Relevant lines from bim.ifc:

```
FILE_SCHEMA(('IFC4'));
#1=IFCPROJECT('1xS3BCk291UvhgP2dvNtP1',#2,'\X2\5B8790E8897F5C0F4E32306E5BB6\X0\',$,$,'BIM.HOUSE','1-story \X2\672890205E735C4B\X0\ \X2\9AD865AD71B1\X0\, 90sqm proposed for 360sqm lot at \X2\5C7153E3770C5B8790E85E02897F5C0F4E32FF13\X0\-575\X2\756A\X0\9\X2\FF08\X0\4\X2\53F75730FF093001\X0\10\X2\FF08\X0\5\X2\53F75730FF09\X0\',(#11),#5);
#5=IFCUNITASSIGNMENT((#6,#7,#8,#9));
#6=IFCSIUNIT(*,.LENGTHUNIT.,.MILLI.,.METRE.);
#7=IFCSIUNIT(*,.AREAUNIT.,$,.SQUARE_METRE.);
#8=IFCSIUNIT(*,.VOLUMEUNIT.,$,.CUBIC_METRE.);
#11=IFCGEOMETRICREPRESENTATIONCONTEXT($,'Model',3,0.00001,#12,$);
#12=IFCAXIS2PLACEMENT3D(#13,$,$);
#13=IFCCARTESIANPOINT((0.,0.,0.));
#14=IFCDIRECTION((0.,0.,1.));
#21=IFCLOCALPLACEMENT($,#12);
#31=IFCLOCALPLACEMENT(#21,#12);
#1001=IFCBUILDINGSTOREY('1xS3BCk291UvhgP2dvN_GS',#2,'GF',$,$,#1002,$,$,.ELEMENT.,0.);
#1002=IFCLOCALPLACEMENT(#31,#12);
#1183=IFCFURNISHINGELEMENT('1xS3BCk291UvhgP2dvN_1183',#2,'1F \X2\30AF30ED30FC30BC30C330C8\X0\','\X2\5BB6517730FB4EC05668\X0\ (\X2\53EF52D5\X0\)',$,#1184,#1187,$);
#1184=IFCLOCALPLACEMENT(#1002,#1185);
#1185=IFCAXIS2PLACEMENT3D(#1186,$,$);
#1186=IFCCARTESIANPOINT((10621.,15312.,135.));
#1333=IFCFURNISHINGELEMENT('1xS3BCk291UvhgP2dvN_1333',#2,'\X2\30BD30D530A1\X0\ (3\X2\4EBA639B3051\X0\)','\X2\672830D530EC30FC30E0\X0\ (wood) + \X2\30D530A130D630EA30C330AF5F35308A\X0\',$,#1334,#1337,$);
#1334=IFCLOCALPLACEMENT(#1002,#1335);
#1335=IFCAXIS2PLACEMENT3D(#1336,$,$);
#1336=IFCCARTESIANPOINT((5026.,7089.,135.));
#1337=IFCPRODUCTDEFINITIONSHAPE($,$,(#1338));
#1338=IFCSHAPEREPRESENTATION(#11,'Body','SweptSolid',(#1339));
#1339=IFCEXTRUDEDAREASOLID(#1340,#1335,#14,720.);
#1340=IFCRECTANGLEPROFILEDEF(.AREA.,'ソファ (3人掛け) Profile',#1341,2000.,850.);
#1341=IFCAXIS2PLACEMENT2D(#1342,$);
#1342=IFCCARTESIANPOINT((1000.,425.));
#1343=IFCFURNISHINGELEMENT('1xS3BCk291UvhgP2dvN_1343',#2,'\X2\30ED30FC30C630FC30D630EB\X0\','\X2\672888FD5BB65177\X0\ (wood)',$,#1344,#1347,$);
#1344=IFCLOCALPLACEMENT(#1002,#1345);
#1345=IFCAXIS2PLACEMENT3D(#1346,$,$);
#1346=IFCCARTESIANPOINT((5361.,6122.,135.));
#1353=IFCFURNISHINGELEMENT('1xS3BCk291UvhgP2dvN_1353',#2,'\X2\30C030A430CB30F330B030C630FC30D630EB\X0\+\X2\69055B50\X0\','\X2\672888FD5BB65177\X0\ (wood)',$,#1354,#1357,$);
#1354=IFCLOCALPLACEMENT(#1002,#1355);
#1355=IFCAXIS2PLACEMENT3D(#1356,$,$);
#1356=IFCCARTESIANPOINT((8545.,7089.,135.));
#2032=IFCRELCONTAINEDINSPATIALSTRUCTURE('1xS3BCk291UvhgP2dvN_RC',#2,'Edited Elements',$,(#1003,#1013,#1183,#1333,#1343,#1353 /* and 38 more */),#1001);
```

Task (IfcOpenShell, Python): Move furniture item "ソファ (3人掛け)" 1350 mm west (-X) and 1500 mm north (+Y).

```python
import ifcopenshell
import ifcopenshell.api.geometry
import ifcopenshell.util.placement
import ifcopenshell.util.unit

model = ifcopenshell.open("bim.ifc")
unit_scale = ifcopenshell.util.unit.calculate_unit_scale(model)

item = model.by_guid("1xS3BCk291UvhgP2dvN_1333")
matrix = ifcopenshell.util.placement.get_local_placement(item.ObjectPlacement)
matrix[0, 3] -= 1.35 / unit_scale
matrix[1, 3] += 1.5 / unit_scale
ifcopenshell.api.geometry.edit_object_placement(model, product=item, matrix=matrix, is_si=False)

print(ifcopenshell.util.placement.get_local_placement(item.ObjectPlacement).round(3) + 0.0)

model.write("bim_v2.ifc")
```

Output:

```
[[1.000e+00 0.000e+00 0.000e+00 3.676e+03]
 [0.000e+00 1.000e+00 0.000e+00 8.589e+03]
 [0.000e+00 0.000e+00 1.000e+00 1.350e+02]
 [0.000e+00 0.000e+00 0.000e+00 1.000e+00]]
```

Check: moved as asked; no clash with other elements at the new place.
